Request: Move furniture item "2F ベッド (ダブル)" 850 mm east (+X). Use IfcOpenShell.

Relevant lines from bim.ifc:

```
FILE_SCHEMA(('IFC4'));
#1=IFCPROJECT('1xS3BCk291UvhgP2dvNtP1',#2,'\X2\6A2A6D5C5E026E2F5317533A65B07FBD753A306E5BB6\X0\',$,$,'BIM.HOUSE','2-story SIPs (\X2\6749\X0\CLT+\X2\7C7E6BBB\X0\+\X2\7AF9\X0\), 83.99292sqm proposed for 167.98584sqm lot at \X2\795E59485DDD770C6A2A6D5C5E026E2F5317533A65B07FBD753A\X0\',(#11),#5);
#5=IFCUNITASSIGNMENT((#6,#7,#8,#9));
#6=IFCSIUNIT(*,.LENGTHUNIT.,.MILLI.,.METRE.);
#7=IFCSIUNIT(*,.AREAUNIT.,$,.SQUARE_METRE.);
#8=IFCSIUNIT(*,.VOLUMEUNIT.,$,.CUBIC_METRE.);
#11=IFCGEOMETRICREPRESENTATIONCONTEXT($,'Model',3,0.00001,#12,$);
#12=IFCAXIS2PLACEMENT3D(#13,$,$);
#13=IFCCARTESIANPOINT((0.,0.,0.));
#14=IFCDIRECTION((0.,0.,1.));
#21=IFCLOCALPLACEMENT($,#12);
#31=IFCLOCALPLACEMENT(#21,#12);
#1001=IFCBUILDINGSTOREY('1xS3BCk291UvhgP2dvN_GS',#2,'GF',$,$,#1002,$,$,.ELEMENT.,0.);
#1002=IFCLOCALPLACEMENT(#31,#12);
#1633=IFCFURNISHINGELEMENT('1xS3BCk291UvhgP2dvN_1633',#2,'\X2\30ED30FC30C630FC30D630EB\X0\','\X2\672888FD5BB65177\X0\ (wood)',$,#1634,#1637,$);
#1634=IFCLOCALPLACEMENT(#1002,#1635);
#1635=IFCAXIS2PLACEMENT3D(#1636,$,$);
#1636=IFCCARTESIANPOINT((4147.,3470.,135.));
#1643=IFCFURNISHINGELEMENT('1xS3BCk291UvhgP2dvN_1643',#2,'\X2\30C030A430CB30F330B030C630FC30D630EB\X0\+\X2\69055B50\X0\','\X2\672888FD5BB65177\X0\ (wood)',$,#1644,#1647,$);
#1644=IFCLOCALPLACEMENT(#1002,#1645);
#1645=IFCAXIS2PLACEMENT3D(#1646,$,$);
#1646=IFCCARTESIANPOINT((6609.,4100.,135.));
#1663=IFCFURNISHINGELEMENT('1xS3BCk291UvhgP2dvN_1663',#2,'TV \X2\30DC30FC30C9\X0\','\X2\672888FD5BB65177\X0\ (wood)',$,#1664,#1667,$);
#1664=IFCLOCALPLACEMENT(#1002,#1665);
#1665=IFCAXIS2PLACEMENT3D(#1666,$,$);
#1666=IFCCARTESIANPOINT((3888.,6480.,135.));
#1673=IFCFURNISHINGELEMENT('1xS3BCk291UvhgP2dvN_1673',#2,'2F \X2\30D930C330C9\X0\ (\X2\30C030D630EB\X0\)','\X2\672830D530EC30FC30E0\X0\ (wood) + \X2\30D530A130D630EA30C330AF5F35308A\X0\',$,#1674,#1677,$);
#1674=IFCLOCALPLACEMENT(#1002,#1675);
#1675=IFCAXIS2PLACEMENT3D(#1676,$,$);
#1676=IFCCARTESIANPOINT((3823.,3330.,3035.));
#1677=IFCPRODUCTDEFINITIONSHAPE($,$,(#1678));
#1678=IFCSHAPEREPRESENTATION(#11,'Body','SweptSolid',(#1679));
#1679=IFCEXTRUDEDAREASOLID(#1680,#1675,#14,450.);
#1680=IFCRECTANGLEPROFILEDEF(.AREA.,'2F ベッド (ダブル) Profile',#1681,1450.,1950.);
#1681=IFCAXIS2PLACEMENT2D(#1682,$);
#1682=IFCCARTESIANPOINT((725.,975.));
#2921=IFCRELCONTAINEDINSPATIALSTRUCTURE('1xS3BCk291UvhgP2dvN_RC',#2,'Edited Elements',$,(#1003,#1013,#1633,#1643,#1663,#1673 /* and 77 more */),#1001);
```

```python
import ifcopenshell
import ifcopenshell.api.geometry
import ifcopenshell.util.placement
import ifcopenshell.util.unit

model = ifcopenshell.open("bim.ifc")
unit_scale = ifcopenshell.util.unit.calculate_unit_scale(model)

item = model.by_id(1673)
matrix = ifcopenshell.util.placement.get_local_placement(item.ObjectPlacement)
matrix[0, 3] += 0.85 / unit_scale
ifcopenshell.api.geometry.edit_object_placement(model, product=item, matrix=matrix, is_si=False)

print(ifcopenshell.util.placement.get_local_placement(item.ObjectPlacement).round(3) + 0.0)

model.write("bim_updated.ifc")
```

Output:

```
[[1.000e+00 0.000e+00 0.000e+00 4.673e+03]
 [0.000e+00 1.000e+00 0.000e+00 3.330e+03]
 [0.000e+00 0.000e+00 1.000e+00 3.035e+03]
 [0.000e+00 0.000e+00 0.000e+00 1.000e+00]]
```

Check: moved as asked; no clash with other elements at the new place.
